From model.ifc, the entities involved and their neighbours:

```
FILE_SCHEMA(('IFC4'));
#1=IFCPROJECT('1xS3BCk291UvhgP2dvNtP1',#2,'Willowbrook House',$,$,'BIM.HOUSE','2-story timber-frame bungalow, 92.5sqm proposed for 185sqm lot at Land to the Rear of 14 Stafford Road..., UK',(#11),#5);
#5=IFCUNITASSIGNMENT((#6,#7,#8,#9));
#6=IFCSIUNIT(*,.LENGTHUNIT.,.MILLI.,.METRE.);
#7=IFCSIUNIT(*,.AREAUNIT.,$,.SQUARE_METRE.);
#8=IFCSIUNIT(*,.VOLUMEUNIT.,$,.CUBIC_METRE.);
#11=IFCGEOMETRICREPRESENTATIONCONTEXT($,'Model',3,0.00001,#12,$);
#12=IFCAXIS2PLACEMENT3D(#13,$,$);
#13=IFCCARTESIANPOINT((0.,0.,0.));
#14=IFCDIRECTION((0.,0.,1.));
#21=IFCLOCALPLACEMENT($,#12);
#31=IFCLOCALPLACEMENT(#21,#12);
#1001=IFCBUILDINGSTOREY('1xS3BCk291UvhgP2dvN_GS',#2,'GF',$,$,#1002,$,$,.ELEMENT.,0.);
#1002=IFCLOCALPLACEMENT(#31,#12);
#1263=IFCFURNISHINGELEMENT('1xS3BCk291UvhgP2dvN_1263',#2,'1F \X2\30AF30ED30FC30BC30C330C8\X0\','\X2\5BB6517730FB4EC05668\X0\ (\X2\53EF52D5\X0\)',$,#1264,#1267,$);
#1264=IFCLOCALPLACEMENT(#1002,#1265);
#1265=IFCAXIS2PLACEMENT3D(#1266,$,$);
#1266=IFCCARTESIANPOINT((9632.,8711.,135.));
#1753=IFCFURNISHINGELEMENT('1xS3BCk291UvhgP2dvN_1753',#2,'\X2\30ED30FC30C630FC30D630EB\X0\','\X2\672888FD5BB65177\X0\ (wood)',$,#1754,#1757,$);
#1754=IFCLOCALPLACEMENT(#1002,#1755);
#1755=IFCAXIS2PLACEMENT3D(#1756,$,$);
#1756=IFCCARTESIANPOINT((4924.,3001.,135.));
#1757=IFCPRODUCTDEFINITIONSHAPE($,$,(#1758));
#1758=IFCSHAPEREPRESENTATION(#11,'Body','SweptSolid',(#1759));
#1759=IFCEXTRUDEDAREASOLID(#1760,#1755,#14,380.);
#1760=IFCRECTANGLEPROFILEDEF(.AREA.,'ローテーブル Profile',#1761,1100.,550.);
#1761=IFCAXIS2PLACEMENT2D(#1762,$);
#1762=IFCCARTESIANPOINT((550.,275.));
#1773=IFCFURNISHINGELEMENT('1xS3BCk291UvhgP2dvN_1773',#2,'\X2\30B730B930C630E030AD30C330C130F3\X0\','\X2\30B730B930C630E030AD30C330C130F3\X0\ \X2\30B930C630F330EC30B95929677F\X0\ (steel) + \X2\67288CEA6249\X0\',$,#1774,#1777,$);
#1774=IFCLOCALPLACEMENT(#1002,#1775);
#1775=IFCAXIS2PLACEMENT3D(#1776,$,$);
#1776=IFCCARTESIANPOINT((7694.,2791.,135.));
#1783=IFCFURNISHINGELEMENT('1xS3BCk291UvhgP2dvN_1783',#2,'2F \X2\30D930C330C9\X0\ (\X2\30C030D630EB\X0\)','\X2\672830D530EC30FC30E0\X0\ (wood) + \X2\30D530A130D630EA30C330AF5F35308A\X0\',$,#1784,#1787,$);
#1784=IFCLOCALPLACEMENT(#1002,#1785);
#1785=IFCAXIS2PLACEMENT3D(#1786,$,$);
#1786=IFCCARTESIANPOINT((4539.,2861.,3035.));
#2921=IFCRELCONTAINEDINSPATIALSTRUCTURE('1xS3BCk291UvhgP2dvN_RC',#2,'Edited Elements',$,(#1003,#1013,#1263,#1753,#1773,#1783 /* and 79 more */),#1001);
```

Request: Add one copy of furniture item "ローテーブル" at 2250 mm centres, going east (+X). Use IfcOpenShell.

```python
import numpy as np
import ifcopenshell
import ifcopenshell.api.geometry
import ifcopenshell.api.root
import ifcopenshell.util.element
import ifcopenshell.util.placement
import ifcopenshell.util.unit

model = ifcopenshell.open("model.ifc")
unit_scale = ifcopenshell.util.unit.calculate_unit_scale(model)


def reuse_history(source, copy):
    """copy_class also copies each property set's owner history, people and application; keep the originals."""
    for rel in copy.IsDefinedBy:
        if rel.is_a("IfcRelDefinesByProperties") and (history := rel.RelatingPropertyDefinition.OwnerHistory):
            rel.RelatingPropertyDefinition.OwnerHistory = source.OwnerHistory
            ifcopenshell.util.element.remove_deep2(model, history)


source = model.by_id(1753)
base = ifcopenshell.util.placement.get_local_placement(source.ObjectPlacement)
step = np.array([1.0, 0.0, 0.0]) * 2.25 / unit_scale

for i in range(1, 2):
    copy = ifcopenshell.api.root.copy_class(model, product=source)
    copy.Representation = ifcopenshell.util.element.copy_deep(
        model, source.Representation, exclude=["IfcGeometricRepresentationContext", "IfcRepresentationMap"]
    )
    reuse_history(source, copy)
    matrix = base.copy()
    matrix[:3, 3] += i * step
    print("added at", matrix[:3, 3].round(3) + 0.0)
    ifcopenshell.api.geometry.edit_object_placement(model, product=copy, matrix=matrix, is_si=False)

model.write("model_updated.ifc")
```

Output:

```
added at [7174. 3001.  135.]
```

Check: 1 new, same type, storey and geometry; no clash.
